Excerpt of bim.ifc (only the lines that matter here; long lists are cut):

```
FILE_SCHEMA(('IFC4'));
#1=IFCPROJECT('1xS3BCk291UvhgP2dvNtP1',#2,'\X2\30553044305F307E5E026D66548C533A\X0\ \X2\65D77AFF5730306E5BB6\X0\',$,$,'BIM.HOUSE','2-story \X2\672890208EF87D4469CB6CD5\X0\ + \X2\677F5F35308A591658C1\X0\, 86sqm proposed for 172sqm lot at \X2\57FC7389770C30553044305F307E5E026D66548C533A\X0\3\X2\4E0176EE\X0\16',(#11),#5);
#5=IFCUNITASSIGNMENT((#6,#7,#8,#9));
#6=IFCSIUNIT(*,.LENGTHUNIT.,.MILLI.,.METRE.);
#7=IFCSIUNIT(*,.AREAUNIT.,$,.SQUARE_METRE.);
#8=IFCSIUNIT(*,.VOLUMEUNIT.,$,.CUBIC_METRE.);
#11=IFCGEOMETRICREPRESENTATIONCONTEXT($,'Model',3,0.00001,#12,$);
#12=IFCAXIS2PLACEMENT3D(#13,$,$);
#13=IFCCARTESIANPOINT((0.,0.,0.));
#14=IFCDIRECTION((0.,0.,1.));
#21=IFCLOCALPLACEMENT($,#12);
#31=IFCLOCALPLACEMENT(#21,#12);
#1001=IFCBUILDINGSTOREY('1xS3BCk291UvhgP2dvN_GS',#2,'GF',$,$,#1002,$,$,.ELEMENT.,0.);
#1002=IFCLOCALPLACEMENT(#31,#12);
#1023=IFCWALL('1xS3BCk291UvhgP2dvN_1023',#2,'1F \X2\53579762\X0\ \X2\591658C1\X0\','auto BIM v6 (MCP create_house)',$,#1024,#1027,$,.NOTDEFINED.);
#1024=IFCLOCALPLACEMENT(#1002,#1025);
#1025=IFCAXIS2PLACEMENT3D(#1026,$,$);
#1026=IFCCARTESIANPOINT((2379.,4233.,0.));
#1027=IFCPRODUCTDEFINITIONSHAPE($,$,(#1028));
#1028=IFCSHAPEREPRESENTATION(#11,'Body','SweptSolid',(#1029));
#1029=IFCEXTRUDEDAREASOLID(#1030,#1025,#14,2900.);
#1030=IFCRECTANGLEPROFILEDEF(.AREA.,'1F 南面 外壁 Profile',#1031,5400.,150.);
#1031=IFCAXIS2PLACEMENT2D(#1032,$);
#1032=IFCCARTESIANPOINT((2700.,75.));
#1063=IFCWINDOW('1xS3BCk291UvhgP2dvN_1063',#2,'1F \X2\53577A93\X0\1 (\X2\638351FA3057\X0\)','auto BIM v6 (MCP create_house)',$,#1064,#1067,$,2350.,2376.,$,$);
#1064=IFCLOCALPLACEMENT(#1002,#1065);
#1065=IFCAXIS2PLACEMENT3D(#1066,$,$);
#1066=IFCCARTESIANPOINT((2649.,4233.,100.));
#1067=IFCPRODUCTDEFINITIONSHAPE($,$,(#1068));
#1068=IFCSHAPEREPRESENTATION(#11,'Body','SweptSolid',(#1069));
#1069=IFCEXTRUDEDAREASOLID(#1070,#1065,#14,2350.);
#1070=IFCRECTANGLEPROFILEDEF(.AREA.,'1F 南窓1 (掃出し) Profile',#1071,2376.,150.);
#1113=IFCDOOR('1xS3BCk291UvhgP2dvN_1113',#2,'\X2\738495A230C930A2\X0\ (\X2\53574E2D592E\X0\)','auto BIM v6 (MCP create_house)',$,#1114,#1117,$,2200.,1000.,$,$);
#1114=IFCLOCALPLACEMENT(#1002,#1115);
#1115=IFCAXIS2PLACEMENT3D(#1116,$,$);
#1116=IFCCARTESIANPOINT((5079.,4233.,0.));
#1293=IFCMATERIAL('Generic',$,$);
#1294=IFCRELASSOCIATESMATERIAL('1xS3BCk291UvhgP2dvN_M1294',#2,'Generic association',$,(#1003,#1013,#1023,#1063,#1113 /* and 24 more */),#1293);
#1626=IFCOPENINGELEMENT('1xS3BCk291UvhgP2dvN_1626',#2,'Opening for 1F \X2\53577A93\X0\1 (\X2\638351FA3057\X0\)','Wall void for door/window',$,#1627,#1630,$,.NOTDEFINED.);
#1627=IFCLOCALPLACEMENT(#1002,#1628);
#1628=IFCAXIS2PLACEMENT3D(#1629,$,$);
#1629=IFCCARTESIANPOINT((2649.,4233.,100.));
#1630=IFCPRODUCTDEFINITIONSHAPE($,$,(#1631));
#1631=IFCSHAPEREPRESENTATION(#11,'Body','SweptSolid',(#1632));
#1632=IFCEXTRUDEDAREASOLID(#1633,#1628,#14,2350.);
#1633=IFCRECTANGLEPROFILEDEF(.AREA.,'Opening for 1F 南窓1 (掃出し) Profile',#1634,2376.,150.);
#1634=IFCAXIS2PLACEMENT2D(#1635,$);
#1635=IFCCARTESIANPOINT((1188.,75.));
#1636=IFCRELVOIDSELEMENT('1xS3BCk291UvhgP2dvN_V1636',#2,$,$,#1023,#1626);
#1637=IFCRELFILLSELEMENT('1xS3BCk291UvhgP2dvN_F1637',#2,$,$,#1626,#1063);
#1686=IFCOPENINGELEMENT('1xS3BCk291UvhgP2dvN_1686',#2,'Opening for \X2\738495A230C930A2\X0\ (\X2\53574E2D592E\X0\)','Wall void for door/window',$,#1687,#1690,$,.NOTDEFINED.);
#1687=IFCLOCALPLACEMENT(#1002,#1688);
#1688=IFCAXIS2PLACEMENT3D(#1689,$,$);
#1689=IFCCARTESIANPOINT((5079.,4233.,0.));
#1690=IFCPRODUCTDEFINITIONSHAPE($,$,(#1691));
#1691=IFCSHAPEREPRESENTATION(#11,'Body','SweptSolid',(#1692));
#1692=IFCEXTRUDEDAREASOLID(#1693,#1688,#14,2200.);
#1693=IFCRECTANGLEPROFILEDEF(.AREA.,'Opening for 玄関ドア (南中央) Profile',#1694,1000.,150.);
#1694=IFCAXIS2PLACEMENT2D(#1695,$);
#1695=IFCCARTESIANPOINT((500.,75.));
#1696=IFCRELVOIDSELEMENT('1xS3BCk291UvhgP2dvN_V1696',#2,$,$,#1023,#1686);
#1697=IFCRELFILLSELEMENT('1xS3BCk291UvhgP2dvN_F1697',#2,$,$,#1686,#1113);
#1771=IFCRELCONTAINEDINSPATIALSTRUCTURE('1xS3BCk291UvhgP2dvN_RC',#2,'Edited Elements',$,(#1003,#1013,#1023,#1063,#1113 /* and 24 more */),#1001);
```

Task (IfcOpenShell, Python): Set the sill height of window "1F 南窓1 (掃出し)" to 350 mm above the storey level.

```python
import numpy as np
import ifcopenshell
import ifcopenshell.api.geometry
import ifcopenshell.geom
import ifcopenshell.util.element
import ifcopenshell.util.placement
import ifcopenshell.util.shape
import ifcopenshell.util.unit

model = ifcopenshell.open("bim.ifc")
unit_scale = ifcopenshell.util.unit.calculate_unit_scale(model)

window = model.by_id(1063)
opening = window.FillsVoids[0].RelatingOpeningElement
storey = ifcopenshell.util.element.get_container(window, ifc_class="IfcBuildingStorey")
level = ifcopenshell.util.placement.get_local_placement(storey.ObjectPlacement)[2, 3]

# The opening's origin need not be at the sill, so measure its lowest point.
shape = ifcopenshell.geom.create_shape(ifcopenshell.geom.settings(), opening)
bottom = ifcopenshell.util.shape.get_shape_bottom_elevation(shape, shape.geometry) / unit_scale
dz = level + 0.35 / unit_scale - bottom

shift = np.array([0.0, 0.0, dz])
# The window is not placed relative to its opening, so move both.
for product in (opening, window):
    matrix = ifcopenshell.util.placement.get_local_placement(product.ObjectPlacement)
    matrix[:3, 3] += shift
    ifcopenshell.api.geometry.edit_object_placement(model, product=product, matrix=matrix, is_si=False)

print(f"moved by {dz * unit_scale:+.3f} m")

model.write("bim_rev.ifc")
```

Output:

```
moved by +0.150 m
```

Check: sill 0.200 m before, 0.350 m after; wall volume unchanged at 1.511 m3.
